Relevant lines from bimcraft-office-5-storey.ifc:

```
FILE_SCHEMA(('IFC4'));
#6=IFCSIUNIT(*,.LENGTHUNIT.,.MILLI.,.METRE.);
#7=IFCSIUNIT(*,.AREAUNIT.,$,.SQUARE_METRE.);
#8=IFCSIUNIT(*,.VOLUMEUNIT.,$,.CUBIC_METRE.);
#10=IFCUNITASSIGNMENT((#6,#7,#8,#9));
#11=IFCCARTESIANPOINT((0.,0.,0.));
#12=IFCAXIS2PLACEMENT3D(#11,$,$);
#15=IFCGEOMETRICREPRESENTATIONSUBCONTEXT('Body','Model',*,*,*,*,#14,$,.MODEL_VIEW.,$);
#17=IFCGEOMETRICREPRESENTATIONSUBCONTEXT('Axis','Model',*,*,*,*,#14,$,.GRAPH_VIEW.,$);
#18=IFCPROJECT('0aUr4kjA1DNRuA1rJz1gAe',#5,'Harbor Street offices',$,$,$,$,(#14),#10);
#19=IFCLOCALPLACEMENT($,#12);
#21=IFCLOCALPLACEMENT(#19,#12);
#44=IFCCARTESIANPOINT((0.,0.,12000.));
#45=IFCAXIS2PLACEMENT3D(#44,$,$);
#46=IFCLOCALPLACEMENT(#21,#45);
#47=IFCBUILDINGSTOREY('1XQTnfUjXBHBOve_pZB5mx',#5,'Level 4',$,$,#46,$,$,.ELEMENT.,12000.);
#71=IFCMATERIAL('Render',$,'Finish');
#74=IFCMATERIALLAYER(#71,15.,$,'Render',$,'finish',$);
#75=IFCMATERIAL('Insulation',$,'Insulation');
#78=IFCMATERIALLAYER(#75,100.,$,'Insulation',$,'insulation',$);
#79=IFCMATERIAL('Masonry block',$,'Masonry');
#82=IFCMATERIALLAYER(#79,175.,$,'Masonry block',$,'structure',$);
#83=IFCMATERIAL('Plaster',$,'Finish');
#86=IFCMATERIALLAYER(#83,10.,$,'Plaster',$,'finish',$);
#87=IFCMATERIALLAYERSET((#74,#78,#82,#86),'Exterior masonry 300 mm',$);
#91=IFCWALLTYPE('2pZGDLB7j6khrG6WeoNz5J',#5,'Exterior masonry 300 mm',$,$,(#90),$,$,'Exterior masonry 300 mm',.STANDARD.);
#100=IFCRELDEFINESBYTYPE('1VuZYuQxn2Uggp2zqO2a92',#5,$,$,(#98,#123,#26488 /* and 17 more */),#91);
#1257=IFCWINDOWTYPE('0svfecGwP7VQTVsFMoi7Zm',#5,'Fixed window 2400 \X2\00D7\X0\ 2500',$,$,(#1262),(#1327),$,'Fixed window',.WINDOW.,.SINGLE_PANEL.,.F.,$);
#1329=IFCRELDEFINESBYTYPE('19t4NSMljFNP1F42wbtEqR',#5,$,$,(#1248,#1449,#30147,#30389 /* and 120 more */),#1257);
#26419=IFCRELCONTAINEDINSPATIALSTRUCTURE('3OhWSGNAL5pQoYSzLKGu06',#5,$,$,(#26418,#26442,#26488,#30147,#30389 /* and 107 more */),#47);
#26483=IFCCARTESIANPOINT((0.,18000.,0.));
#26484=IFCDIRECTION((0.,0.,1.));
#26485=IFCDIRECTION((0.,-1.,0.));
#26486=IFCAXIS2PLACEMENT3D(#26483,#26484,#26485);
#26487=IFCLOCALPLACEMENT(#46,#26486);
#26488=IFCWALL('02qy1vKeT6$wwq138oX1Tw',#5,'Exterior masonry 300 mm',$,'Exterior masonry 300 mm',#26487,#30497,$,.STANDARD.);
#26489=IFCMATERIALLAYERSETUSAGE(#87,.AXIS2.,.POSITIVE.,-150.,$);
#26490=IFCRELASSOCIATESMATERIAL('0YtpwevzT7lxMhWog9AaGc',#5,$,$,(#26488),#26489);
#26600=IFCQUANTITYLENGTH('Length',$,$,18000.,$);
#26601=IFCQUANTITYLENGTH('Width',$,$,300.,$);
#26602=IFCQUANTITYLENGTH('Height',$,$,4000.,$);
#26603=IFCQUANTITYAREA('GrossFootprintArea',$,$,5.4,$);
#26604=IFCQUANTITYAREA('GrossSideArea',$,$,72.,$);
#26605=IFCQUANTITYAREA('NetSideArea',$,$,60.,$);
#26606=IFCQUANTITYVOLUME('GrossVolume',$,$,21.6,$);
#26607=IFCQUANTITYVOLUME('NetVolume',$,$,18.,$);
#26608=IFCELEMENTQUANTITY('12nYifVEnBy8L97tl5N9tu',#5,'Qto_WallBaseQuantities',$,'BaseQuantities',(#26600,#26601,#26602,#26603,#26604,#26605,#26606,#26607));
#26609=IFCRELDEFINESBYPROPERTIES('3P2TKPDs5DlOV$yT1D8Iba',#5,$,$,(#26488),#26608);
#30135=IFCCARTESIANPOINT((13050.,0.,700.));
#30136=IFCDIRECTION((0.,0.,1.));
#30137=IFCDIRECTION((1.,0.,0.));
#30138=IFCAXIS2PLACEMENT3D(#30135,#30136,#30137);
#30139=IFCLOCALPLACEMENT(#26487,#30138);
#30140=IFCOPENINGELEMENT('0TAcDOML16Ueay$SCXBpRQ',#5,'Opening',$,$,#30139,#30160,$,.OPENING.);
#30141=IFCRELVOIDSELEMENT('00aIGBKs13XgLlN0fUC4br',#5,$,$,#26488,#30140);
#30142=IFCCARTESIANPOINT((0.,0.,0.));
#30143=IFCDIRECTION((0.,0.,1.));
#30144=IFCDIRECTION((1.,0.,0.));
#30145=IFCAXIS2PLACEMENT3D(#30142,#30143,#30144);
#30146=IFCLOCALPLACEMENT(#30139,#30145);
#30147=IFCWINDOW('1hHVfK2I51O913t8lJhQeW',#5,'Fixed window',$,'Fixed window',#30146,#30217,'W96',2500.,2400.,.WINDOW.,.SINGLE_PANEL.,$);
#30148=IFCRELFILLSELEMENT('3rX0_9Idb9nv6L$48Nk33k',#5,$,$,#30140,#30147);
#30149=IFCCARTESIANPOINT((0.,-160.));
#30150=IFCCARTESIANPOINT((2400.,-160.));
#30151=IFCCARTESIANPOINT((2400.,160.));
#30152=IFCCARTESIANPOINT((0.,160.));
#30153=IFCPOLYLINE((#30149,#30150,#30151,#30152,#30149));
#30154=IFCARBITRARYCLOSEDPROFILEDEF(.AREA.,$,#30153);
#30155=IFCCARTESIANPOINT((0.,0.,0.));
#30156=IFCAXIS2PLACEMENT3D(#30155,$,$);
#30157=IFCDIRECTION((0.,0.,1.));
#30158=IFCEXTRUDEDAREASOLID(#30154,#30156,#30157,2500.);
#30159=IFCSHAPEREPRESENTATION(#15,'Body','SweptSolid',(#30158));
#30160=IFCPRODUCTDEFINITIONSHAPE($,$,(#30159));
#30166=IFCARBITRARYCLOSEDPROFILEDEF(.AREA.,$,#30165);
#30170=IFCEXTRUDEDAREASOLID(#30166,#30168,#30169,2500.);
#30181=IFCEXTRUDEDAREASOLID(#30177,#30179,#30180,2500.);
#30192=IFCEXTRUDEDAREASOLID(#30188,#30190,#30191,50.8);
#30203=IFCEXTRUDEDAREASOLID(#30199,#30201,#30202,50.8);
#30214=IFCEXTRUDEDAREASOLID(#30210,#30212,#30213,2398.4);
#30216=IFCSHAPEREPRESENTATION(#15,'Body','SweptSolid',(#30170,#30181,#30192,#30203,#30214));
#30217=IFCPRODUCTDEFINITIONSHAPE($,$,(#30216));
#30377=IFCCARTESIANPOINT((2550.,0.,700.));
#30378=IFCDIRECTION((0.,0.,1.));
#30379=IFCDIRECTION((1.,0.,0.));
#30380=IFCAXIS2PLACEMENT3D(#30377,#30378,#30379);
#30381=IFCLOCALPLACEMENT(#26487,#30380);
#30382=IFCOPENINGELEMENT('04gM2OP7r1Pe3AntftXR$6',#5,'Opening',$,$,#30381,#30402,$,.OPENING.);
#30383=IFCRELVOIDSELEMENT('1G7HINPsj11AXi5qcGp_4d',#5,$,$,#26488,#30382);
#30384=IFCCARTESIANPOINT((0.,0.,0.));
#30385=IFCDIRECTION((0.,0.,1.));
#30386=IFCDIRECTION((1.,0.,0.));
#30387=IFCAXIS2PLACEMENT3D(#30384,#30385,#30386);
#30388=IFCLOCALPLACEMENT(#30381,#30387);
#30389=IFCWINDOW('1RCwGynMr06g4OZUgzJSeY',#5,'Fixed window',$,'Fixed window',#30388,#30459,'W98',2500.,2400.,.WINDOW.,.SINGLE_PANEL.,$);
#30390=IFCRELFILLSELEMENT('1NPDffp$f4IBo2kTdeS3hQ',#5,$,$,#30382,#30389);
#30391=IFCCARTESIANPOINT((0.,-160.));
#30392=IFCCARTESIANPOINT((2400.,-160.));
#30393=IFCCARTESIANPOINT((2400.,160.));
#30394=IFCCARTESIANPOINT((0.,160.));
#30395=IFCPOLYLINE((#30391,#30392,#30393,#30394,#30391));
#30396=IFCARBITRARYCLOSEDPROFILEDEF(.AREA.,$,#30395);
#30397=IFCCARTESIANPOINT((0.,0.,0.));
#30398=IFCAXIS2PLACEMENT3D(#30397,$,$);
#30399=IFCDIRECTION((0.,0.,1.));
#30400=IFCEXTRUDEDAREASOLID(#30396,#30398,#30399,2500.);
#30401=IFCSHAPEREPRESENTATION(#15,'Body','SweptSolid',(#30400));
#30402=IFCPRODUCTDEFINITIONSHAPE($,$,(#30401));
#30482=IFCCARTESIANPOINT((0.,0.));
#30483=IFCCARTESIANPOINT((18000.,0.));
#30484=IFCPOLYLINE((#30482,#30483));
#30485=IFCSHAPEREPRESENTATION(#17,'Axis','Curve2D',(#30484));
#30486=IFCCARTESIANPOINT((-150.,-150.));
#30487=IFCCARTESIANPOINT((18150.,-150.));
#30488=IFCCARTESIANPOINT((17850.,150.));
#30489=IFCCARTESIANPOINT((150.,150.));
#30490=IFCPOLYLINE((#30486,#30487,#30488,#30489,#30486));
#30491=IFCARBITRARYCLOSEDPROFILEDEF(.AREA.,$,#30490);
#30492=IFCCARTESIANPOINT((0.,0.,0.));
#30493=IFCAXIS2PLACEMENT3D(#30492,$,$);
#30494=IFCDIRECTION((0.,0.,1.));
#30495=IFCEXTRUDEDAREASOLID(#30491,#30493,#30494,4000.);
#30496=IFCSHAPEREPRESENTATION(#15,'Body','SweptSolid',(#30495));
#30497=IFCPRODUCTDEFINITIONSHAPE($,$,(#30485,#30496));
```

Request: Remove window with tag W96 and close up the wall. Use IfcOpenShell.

```python
import ifcopenshell
import ifcopenshell.api.feature
import ifcopenshell.api.pset
import ifcopenshell.api.root
import ifcopenshell.geom
import ifcopenshell.util.element
import ifcopenshell.util.shape
import ifcopenshell.util.unit

model = ifcopenshell.open("bimcraft-office-5-storey.ifc")
area_scale = ifcopenshell.util.unit.calculate_unit_scale(model, "AREAUNIT")
volume_scale = ifcopenshell.util.unit.calculate_unit_scale(model, "VOLUMEUNIT")
settings = ifcopenshell.geom.settings()


def volume(element):
    """Net volume in cubic metres, openings subtracted."""
    shape = ifcopenshell.geom.create_shape(settings, element)
    return ifcopenshell.util.shape.get_volume(shape.geometry)


window = model.by_guid("1hHVfK2I51O913t8lJhQeW")
opening = window.FillsVoids[0].RelatingOpeningElement
wall = opening.VoidsElements[0].RelatingBuildingElement
before = volume(wall)

ifcopenshell.api.root.remove_product(model, product=window)
ifcopenshell.api.feature.remove_feature(model, feature=opening)

after = volume(wall)
thickness = 0.3  # wall thickness in metres

# Update the wall's stored quantities.
qto = model.by_id(ifcopenshell.util.element.get_pset(wall, "Qto_WallBaseQuantities", should_inherit=False)["id"])
ifcopenshell.api.pset.edit_qto(model, qto=qto, properties={
    "NetSideArea": after / thickness / area_scale,
    "NetVolume": after / volume_scale,
})

print(f"wall volume {before:.3f} -> {after:.3f} m3")

model.write("bimcraft-office-5-storey_v2.ifc")
```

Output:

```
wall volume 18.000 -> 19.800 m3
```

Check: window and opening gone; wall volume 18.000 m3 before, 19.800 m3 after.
